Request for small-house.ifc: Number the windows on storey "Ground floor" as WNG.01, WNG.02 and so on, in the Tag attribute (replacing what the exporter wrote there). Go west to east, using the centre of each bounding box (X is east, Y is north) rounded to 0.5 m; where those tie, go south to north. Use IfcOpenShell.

First a look at what the model holds.

```python
import ifcopenshell
import ifcopenshell.util.element
import ifcopenshell.util.placement

model = ifcopenshell.open("small-house.ifc")
print(model.schema)
storey = next(s for s in model.by_type("IfcBuildingStorey") if s.Name == "Ground floor")
windows = [e for e in ifcopenshell.util.element.get_decomposition(storey) if e.is_a("IfcWindow")]
for e in sorted(windows, key=lambda e: e.id()):
    origin = ifcopenshell.util.placement.get_local_placement(e.ObjectPlacement)[:3, 3]
    print(e.id(), e.Tag, e.Name, origin.round(2) + 0.0, sep=" | ")
```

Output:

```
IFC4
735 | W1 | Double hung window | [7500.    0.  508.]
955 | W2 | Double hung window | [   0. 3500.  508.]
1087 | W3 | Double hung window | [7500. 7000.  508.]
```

```python
import ifcopenshell
import ifcopenshell.geom
import ifcopenshell.util.element
import ifcopenshell.util.shape

model = ifcopenshell.open("small-house.ifc")
settings = ifcopenshell.geom.settings()
settings.set("use-world-coords", True)


def centre(element):
    shape = ifcopenshell.geom.create_shape(settings, element)
    return ifcopenshell.util.shape.get_bbox_centroid(shape.geometry)


storey = next(s for s in model.by_type("IfcBuildingStorey") if s.Name == "Ground floor")
windows = [e for e in ifcopenshell.util.element.get_decomposition(storey) if e.is_a("IfcWindow")]

# Insertion points can sit at a corner or the storey origin, so sort by the geometry (in metres).
centres = {e: centre(e) for e in windows}
windows.sort(key=lambda e: (round(centres[e][0] / 0.5), centres[e][1]))

for i, e in enumerate(windows, start=1):
    number = f"WNG.{i:02d}"
    e.Tag = number
    print(e.id(), number)

model.write("small-house_updated.ifc")
```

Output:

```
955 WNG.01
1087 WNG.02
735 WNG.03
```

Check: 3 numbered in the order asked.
